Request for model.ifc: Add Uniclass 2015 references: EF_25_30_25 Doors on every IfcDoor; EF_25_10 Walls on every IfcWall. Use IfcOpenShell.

First a look at what the model holds.

```python
import ifcopenshell

model = ifcopenshell.open("model.ifc")
print(model.schema)
print("classifications:", [c.Name for c in model.by_type("IfcClassification")])
for ifc_class in ("IfcDoor", "IfcRoof", "IfcStair", "IfcWall", "IfcWindow"):
    print(ifc_class, len(model.by_type(ifc_class)))
```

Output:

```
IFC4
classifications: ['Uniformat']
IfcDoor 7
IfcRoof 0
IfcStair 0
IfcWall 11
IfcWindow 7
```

```python
import ifcopenshell
import ifcopenshell.api.classification

model = ifcopenshell.open("model.ifc")

system = ifcopenshell.api.classification.add_classification(model, classification="Uniclass 2015")

codes = {
    "IfcDoor": ("EF_25_30_25", "Doors"),
    "IfcWall": ("EF_25_10", "Walls"),
}
for ifc_class, (code, name) in codes.items():
    products = model.by_type(ifc_class)
    ifcopenshell.api.classification.add_reference(
        model, products=products, classification=system, identification=code, name=name
    )
    print(code, len(products))

model.write("model_edited.ifc")
```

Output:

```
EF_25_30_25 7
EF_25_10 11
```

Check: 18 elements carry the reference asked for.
